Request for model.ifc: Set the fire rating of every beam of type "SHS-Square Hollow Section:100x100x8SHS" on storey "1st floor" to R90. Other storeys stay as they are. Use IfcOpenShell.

First a look at what the model holds.

```python
import ifcopenshell
import ifcopenshell.util.element

model = ifcopenshell.open("model.ifc")
print(model.schema)
storey = next(s for s in model.by_type("IfcBuildingStorey") if s.Name == "1st floor")
beams = [e for e in ifcopenshell.util.element.get_decomposition(storey) if e.is_a("IfcBeam")]
seen = {}
for e in beams:
    element_type = ifcopenshell.util.element.get_type(e)
    key = (element_type.Name if element_type != e and element_type else None, ifcopenshell.util.element.get_pset(e, "Pset_BeamCommon", "FireRating"))
    seen[key] = seen.get(key, 0) + 1
for (name, value), count in sorted(seen.items(), key=str):
    print(count, "x", name, "|", value)
```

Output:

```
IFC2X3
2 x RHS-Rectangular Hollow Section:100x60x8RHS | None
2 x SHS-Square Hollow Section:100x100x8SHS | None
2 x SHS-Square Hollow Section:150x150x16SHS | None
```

```python
import ifcopenshell
import ifcopenshell.api.pset
import ifcopenshell.util.element

model = ifcopenshell.open("model.ifc")

storey = next(s for s in model.by_type("IfcBuildingStorey") if s.Name == "1st floor")
beams = [e for e in ifcopenshell.util.element.get_decomposition(storey) if e.is_a("IfcBeam")]

count = 0
for e in beams:
    element_type = ifcopenshell.util.element.get_type(e)
    if element_type in (None, e) or element_type.Name != "SHS-Square Hollow Section:100x100x8SHS":
        continue
    # add_pset returns the element's existing set when there is one.
    pset = ifcopenshell.api.pset.add_pset(model, product=e, name="Pset_BeamCommon")
    ifcopenshell.api.pset.edit_pset(model, pset=pset, properties={"FireRating": "R90"})
    count += 1

print(count, "beams updated")

model.write("model_updated.ifc")
```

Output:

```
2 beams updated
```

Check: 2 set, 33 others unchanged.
